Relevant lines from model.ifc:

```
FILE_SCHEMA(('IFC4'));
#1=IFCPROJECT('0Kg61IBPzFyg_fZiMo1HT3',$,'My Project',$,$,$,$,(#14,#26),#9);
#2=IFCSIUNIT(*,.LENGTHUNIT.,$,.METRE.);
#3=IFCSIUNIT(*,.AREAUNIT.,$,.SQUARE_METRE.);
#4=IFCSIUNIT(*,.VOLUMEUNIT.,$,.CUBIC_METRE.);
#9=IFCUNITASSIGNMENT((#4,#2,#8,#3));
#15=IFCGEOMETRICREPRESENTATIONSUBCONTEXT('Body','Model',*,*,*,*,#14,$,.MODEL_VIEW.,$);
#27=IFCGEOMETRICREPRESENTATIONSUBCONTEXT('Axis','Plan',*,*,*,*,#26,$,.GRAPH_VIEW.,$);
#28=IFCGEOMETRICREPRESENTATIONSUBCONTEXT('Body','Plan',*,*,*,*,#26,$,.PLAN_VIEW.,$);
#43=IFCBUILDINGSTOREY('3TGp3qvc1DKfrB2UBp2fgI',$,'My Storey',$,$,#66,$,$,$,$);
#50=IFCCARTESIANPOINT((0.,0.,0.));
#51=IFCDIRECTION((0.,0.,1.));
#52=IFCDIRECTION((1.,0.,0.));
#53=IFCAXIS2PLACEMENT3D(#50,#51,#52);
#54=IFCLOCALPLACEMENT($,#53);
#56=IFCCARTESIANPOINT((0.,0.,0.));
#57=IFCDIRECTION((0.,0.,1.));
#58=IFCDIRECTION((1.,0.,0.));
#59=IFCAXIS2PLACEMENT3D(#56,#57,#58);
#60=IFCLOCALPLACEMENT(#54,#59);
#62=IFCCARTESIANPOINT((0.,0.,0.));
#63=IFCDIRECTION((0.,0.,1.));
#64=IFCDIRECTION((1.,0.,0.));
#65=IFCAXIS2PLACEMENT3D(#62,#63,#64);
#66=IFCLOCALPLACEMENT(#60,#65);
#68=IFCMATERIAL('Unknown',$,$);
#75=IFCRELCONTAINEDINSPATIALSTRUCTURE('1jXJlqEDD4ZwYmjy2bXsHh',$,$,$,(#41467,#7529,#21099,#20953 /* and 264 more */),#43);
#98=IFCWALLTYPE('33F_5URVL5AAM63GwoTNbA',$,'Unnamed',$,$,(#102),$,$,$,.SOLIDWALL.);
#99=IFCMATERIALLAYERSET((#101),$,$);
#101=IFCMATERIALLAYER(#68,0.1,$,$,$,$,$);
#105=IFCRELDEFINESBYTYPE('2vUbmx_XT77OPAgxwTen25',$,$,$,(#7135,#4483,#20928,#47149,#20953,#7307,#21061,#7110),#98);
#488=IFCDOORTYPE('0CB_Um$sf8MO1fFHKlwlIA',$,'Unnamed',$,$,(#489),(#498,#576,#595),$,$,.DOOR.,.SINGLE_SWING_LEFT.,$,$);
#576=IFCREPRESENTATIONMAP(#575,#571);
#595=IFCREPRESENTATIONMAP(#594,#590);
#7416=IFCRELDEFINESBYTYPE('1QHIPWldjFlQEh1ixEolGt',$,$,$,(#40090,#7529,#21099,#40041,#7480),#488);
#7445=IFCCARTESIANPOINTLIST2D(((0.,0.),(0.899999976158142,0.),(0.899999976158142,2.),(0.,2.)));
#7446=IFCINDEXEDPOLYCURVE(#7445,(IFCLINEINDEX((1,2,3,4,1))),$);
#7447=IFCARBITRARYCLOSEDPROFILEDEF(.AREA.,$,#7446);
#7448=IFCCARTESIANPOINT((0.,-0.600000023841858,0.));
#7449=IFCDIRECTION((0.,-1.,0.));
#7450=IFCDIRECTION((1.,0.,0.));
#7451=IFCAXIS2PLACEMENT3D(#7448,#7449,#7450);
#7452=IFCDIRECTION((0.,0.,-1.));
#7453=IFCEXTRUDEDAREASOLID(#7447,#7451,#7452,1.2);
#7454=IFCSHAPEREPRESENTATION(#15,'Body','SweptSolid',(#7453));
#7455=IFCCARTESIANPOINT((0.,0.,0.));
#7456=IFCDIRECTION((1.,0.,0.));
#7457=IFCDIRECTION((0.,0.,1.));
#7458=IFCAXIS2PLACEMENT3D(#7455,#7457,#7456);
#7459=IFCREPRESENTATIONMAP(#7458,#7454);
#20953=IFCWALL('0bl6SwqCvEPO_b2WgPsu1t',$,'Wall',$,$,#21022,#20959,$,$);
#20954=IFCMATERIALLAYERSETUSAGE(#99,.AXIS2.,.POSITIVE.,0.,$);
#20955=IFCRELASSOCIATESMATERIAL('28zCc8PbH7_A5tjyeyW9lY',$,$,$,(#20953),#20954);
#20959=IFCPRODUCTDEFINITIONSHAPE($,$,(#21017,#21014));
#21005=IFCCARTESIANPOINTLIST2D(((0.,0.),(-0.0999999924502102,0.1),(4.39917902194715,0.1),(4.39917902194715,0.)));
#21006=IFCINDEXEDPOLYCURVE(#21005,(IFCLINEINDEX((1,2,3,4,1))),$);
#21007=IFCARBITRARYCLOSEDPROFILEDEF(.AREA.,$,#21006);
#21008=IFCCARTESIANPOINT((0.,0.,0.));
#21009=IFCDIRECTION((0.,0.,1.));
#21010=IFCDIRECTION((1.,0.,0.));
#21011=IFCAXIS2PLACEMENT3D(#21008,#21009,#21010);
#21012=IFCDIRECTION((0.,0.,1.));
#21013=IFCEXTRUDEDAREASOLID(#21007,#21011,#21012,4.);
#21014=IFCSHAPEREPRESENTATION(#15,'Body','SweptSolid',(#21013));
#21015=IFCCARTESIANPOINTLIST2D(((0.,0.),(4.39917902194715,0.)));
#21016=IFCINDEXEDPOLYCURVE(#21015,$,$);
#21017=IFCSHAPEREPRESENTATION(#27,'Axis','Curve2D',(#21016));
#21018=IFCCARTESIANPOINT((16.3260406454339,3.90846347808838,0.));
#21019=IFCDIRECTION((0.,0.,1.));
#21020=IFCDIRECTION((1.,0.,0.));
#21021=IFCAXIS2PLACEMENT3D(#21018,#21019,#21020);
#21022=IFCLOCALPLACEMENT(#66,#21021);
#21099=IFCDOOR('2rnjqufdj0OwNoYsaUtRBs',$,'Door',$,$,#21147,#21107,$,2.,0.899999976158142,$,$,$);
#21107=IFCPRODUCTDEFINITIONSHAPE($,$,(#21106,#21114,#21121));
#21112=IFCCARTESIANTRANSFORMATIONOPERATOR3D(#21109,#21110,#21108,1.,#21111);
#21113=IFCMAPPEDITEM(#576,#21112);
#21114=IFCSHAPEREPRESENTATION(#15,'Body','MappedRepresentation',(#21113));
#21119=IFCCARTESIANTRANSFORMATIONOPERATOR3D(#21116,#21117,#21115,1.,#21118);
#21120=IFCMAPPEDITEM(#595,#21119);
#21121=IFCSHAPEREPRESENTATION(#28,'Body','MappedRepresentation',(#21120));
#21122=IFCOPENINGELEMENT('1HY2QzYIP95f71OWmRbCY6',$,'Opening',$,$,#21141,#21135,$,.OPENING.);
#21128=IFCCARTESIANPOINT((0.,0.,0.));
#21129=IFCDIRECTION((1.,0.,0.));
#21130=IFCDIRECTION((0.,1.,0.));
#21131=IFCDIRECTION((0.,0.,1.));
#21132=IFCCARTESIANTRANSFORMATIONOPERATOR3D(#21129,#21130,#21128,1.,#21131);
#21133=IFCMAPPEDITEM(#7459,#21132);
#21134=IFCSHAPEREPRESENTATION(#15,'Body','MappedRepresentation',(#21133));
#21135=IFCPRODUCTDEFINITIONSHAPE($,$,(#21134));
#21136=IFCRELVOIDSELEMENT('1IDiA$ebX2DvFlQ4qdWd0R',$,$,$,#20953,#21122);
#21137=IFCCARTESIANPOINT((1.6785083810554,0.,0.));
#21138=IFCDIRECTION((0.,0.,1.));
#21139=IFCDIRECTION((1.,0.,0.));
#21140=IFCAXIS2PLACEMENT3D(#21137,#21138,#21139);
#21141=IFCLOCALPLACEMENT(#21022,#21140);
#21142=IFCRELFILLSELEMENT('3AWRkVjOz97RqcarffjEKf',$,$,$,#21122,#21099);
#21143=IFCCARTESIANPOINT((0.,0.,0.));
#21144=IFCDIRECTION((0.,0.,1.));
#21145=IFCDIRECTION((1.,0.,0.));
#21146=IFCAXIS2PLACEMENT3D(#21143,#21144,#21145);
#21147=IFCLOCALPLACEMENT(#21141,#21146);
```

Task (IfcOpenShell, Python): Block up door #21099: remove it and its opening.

```python
import ifcopenshell
import ifcopenshell.api.feature
import ifcopenshell.api.root
import ifcopenshell.geom
import ifcopenshell.util.shape

model = ifcopenshell.open("model.ifc")
settings = ifcopenshell.geom.settings()


def volume(element):
    """Net volume in cubic metres, openings subtracted."""
    shape = ifcopenshell.geom.create_shape(settings, element)
    return ifcopenshell.util.shape.get_volume(shape.geometry)


door = model.by_id(21099)
opening = door.FillsVoids[0].RelatingOpeningElement
wall = opening.VoidsElements[0].RelatingBuildingElement
before = volume(wall)

ifcopenshell.api.root.remove_product(model, product=door)
ifcopenshell.api.feature.remove_feature(model, feature=opening)

after = volume(wall)

print(f"wall volume {before:.3f} -> {after:.3f} m3")

model.write("model-out.ifc")
```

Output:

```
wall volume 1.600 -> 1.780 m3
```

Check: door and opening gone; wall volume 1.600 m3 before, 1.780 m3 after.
